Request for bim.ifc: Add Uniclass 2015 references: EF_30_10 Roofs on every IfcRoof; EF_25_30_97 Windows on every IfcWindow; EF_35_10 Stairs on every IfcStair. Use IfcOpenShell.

First a look at what the model holds.

```python
import ifcopenshell

model = ifcopenshell.open("bim.ifc")
print(model.schema)
print("classifications:", [c.Name for c in model.by_type("IfcClassification")])
for ifc_class in ("IfcDoor", "IfcRoof", "IfcStair", "IfcWall", "IfcWindow"):
    print(ifc_class, len(model.by_type(ifc_class)))
```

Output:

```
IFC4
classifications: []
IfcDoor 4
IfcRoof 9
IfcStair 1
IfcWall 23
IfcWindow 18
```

```python
import ifcopenshell
import ifcopenshell.api.classification

model = ifcopenshell.open("bim.ifc")

system = ifcopenshell.api.classification.add_classification(model, classification="Uniclass 2015")

codes = {
    "IfcRoof": ("EF_30_10", "Roofs"),
    "IfcWindow": ("EF_25_30_97", "Windows"),
    "IfcStair": ("EF_35_10", "Stairs"),
}
for ifc_class, (code, name) in codes.items():
    products = model.by_type(ifc_class)
    ifcopenshell.api.classification.add_reference(
        model, products=products, classification=system, identification=code, name=name
    )
    print(code, len(products))

model.write("bim_rev.ifc")
```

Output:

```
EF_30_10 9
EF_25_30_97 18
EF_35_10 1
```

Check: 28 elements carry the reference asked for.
